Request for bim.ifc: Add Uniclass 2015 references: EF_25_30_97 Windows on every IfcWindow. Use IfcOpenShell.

First a look at what the model holds.

```python
import ifcopenshell

model = ifcopenshell.open("bim.ifc")
print(model.schema)
print("classifications:", [c.Name for c in model.by_type("IfcClassification")])
for ifc_class in ("IfcDoor", "IfcRoof", "IfcStair", "IfcWall", "IfcWindow"):
    print(ifc_class, len(model.by_type(ifc_class)))
```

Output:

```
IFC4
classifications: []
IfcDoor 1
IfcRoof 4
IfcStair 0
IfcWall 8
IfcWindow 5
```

```python
import ifcopenshell
import ifcopenshell.api.classification

model = ifcopenshell.open("bim.ifc")

system = ifcopenshell.api.classification.add_classification(model, classification="Uniclass 2015")

codes = {
    "IfcWindow": ("EF_25_30_97", "Windows"),
}
for ifc_class, (code, name) in codes.items():
    products = model.by_type(ifc_class)
    ifcopenshell.api.classification.add_reference(
        model, products=products, classification=system, identification=code, name=name
    )
    print(code, len(products))

model.write("bim_v2.ifc")
```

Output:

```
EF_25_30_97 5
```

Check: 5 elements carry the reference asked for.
